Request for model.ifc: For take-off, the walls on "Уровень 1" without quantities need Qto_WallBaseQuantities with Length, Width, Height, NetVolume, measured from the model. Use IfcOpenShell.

First a look at what the model holds.

```python
import ifcopenshell
import ifcopenshell.util.element
import ifcopenshell.util.unit

model = ifcopenshell.open("model.ifc")
print(model.schema)
for unit_type in ("LENGTHUNIT", "AREAUNIT", "VOLUMEUNIT"):
    print(unit_type, ifcopenshell.util.unit.calculate_unit_scale(model, unit_type))
storey = next(s for s in model.by_type("IfcBuildingStorey") if s.Name == "Уровень 1")
walls = [e for e in ifcopenshell.util.element.get_decomposition(storey) if e.is_a("IfcWall")]
for e in sorted(walls, key=lambda e: e.id()):
    print(e.id(), e.is_a(), e.Name, list(ifcopenshell.util.element.get_psets(e, qtos_only=True)), sep=" | ")
```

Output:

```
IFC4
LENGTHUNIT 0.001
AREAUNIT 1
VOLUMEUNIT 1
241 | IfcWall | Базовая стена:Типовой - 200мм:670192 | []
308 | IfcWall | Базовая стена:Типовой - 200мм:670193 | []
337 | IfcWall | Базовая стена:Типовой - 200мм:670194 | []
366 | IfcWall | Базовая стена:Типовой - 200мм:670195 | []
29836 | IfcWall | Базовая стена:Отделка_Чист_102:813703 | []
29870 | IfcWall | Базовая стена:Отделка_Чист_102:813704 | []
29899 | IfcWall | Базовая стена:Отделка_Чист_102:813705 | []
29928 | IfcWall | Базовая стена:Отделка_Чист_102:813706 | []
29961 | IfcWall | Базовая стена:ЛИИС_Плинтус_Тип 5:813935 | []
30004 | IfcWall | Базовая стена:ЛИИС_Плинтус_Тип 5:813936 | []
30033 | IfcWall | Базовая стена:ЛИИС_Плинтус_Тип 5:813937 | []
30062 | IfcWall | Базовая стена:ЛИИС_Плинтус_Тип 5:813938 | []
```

```python
import ifcopenshell
import ifcopenshell.api.pset
import ifcopenshell.geom
import ifcopenshell.util.element
import ifcopenshell.util.shape
import ifcopenshell.util.unit

model = ifcopenshell.open("model.ifc")
unit_scale = ifcopenshell.util.unit.calculate_unit_scale(model)
volume_scale = ifcopenshell.util.unit.calculate_unit_scale(model, "VOLUMEUNIT")
settings = ifcopenshell.geom.settings()

storey = next(s for s in model.by_type("IfcBuildingStorey") if s.Name == "Уровень 1")
walls = [e for e in ifcopenshell.util.element.get_decomposition(storey) if e.is_a("IfcWall")]

for e in sorted(walls, key=lambda e: e.id()):
    if ifcopenshell.util.element.get_psets(e, qtos_only=True, should_inherit=False):
        continue
    # Geometry comes back in metres, in the element's own axes.
    shape = ifcopenshell.geom.create_shape(settings, e)
    values = {
        "Length": ifcopenshell.util.shape.get_x(shape.geometry) / unit_scale,
        "Width": ifcopenshell.util.shape.get_y(shape.geometry) / unit_scale,
        "Height": ifcopenshell.util.shape.get_z(shape.geometry) / unit_scale,
        "NetVolume": ifcopenshell.util.shape.get_volume(shape.geometry) / volume_scale,
    }
    qto = ifcopenshell.api.pset.add_qto(model, product=e, name="Qto_WallBaseQuantities")
    ifcopenshell.api.pset.edit_qto(model, qto=qto, properties=values)
    print(e.id(), {k: round(v, 3) for k, v in values.items()})

model.write("model_updated.ifc")
```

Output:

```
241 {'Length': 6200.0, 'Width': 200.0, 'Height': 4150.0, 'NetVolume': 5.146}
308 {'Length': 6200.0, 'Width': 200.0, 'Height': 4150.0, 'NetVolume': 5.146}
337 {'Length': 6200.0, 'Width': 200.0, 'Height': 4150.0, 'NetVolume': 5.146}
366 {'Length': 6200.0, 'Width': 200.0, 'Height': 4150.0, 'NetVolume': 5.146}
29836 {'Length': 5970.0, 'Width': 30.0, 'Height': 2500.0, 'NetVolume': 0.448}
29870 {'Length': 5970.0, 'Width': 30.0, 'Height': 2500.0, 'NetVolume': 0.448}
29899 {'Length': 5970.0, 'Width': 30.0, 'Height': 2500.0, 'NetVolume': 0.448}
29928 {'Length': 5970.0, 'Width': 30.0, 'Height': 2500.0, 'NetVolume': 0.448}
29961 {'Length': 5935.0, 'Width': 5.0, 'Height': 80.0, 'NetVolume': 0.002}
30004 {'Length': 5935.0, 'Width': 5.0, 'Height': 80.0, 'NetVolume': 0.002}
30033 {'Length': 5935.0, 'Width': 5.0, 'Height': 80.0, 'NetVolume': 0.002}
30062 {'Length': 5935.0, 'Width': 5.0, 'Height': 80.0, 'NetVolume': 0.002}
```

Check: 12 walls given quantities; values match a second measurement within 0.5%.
